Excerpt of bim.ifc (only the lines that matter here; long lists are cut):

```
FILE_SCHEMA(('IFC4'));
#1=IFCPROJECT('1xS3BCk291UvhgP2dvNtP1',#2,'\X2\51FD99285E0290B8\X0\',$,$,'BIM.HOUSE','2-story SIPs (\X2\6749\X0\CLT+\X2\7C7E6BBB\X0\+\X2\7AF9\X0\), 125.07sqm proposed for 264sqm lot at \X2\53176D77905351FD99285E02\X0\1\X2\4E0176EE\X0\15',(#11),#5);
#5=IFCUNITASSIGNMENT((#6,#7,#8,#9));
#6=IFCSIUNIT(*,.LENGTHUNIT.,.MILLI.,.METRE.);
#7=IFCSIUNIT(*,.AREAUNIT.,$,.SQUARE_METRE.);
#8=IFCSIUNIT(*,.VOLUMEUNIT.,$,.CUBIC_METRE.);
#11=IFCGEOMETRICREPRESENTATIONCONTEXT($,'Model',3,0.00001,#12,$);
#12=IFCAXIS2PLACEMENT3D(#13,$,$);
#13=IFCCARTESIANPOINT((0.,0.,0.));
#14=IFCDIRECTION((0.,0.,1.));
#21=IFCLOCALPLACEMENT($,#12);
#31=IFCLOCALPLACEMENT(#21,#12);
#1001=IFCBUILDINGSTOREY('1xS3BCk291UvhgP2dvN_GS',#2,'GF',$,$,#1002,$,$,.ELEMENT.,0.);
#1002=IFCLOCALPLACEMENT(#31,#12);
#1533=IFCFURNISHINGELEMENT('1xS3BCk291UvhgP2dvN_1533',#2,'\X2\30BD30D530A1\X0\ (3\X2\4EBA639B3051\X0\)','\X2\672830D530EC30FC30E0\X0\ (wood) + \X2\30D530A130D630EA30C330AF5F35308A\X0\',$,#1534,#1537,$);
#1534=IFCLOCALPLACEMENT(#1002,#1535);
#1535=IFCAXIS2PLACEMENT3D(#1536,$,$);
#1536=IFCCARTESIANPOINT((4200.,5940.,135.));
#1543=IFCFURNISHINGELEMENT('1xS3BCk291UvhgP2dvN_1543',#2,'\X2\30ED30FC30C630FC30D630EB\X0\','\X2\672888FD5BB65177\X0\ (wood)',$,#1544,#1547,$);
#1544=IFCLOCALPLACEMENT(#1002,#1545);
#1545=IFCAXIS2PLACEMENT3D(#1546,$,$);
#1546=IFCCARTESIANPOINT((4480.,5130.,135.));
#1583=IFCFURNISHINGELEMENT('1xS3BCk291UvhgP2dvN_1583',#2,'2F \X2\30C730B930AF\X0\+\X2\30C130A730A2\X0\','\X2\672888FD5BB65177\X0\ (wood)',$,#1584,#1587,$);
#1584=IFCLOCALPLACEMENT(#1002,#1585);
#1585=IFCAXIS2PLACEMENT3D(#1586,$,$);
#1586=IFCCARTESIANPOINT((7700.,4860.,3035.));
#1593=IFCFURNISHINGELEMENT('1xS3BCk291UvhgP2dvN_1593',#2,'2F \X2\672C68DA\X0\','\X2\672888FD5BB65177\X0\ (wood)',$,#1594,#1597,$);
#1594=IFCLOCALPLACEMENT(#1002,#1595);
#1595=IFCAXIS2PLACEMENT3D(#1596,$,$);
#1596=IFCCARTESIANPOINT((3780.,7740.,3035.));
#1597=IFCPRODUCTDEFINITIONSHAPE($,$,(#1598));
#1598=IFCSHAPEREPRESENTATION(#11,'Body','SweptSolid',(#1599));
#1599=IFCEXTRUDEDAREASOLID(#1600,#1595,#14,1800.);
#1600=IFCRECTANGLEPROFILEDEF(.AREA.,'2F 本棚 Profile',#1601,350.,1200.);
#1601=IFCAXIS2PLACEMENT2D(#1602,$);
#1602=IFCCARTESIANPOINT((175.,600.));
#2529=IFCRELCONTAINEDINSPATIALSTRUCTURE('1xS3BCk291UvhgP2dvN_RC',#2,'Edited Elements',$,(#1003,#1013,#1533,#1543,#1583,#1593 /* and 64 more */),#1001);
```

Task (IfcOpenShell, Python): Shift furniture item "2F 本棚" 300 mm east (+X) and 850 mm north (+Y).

```python
import ifcopenshell
import ifcopenshell.api.geometry
import ifcopenshell.util.placement

model = ifcopenshell.open("bim.ifc")

item = model.by_guid("1xS3BCk291UvhgP2dvN_1593")
matrix = ifcopenshell.util.placement.get_local_placement(item.ObjectPlacement)
matrix[0, 3] += 300.0
matrix[1, 3] += 850.0
ifcopenshell.api.geometry.edit_object_placement(model, product=item, matrix=matrix, is_si=False)

print(ifcopenshell.util.placement.get_local_placement(item.ObjectPlacement).round(3) + 0.0)

model.write("bim_v2.ifc")
```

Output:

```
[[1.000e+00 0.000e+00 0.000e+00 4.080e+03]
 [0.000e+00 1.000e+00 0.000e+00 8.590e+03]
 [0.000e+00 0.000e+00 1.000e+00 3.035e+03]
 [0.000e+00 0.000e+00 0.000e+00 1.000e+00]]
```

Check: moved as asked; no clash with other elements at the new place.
